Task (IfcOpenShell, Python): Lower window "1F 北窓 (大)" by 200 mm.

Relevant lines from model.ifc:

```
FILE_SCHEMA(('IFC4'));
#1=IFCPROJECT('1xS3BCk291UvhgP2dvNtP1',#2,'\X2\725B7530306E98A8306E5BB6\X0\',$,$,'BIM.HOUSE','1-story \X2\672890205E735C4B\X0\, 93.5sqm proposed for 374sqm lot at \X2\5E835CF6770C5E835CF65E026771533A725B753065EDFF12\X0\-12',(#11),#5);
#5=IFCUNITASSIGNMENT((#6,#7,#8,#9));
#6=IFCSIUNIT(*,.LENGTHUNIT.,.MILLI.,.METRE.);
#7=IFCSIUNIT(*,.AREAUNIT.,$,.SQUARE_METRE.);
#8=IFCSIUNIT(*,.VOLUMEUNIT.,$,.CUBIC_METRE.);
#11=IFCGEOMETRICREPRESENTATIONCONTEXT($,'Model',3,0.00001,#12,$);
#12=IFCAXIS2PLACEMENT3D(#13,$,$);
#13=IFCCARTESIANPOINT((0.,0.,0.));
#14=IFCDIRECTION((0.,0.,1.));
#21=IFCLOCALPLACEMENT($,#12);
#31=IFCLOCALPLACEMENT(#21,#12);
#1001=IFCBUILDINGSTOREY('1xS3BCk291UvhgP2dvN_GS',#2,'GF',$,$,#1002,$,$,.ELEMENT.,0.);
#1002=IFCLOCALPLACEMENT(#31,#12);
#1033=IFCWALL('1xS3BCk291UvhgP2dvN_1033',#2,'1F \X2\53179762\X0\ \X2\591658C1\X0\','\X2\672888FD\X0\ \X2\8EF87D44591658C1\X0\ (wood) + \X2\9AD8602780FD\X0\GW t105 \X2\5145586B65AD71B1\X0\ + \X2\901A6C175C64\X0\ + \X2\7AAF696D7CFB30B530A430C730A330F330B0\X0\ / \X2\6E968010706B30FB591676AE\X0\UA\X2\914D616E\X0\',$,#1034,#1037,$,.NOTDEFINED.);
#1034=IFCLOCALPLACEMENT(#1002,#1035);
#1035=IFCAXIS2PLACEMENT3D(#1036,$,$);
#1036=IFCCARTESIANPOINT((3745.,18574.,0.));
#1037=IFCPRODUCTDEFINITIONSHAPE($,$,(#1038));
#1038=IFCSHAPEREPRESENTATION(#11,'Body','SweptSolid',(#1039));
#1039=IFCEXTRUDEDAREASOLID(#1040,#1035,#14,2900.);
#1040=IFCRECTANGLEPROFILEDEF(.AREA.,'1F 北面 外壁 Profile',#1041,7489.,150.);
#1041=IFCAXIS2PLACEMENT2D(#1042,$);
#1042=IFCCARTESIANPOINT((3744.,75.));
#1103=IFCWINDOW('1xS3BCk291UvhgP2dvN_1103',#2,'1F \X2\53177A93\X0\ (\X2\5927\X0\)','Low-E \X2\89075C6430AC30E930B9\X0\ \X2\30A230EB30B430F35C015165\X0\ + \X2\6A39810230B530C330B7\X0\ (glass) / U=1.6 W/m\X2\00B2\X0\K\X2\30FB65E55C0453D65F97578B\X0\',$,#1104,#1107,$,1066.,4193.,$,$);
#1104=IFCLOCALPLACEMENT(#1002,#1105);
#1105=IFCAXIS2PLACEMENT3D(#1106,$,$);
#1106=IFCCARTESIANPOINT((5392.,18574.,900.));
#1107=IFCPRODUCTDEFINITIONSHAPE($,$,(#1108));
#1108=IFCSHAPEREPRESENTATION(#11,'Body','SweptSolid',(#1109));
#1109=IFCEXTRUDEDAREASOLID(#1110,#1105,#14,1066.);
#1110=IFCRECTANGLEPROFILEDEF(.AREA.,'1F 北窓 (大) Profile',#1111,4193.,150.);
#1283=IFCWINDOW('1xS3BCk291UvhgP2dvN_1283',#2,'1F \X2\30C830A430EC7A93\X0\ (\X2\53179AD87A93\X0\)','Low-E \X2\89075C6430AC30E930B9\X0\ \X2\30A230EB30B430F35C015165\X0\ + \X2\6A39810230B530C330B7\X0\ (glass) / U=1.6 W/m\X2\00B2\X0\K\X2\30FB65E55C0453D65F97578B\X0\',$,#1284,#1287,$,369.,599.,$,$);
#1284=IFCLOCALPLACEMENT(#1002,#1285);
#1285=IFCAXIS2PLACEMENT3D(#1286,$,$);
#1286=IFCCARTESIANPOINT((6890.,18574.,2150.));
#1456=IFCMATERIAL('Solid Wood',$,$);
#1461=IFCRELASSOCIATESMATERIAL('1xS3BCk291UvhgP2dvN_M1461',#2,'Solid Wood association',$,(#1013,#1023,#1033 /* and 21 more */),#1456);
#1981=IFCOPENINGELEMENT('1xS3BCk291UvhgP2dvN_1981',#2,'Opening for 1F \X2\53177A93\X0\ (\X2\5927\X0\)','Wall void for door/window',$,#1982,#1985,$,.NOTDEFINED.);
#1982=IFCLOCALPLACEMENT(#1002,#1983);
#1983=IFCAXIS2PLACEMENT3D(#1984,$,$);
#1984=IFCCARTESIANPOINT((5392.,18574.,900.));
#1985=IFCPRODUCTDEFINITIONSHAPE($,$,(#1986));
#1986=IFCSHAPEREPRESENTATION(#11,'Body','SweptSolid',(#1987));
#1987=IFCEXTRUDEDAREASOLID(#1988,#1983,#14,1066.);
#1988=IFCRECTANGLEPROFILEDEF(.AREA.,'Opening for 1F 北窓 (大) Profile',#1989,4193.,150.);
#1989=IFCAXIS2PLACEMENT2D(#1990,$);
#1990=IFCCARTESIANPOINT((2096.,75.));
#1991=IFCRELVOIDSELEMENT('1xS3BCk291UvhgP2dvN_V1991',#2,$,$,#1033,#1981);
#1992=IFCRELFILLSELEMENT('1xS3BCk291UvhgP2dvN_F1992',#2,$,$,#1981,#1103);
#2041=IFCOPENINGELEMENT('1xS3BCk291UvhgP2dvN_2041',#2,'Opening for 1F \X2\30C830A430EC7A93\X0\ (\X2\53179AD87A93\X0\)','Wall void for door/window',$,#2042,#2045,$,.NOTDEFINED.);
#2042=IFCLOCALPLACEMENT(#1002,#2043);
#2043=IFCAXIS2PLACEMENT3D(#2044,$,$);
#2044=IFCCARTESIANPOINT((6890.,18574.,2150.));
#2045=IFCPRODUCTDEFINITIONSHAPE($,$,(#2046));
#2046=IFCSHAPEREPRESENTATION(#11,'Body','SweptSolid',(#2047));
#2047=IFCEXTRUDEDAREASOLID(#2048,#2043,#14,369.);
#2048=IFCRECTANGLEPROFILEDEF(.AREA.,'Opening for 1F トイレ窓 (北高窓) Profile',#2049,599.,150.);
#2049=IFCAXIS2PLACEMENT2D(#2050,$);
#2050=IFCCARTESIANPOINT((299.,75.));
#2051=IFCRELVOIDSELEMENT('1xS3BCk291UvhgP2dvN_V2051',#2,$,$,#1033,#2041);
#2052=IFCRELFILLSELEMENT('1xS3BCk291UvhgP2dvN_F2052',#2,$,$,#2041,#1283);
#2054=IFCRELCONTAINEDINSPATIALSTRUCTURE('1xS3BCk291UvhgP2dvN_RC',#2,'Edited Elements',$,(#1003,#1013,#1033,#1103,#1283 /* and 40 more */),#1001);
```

```python
import numpy as np
import ifcopenshell
import ifcopenshell.api.geometry
import ifcopenshell.util.placement
import ifcopenshell.util.unit

model = ifcopenshell.open("model.ifc")
unit_scale = ifcopenshell.util.unit.calculate_unit_scale(model)

window = model.by_guid("1xS3BCk291UvhgP2dvN_1103")
opening = window.FillsVoids[0].RelatingOpeningElement
dz = -0.2 / unit_scale

shift = np.array([0.0, 0.0, dz])
# The window is not placed relative to its opening, so move both.
for product in (opening, window):
    matrix = ifcopenshell.util.placement.get_local_placement(product.ObjectPlacement)
    matrix[:3, 3] += shift
    ifcopenshell.api.geometry.edit_object_placement(model, product=product, matrix=matrix, is_si=False)

print(f"moved by {dz * unit_scale:+.3f} m")

model.write("model_updated.ifc")
```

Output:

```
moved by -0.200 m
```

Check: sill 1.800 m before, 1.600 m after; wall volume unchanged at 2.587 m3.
